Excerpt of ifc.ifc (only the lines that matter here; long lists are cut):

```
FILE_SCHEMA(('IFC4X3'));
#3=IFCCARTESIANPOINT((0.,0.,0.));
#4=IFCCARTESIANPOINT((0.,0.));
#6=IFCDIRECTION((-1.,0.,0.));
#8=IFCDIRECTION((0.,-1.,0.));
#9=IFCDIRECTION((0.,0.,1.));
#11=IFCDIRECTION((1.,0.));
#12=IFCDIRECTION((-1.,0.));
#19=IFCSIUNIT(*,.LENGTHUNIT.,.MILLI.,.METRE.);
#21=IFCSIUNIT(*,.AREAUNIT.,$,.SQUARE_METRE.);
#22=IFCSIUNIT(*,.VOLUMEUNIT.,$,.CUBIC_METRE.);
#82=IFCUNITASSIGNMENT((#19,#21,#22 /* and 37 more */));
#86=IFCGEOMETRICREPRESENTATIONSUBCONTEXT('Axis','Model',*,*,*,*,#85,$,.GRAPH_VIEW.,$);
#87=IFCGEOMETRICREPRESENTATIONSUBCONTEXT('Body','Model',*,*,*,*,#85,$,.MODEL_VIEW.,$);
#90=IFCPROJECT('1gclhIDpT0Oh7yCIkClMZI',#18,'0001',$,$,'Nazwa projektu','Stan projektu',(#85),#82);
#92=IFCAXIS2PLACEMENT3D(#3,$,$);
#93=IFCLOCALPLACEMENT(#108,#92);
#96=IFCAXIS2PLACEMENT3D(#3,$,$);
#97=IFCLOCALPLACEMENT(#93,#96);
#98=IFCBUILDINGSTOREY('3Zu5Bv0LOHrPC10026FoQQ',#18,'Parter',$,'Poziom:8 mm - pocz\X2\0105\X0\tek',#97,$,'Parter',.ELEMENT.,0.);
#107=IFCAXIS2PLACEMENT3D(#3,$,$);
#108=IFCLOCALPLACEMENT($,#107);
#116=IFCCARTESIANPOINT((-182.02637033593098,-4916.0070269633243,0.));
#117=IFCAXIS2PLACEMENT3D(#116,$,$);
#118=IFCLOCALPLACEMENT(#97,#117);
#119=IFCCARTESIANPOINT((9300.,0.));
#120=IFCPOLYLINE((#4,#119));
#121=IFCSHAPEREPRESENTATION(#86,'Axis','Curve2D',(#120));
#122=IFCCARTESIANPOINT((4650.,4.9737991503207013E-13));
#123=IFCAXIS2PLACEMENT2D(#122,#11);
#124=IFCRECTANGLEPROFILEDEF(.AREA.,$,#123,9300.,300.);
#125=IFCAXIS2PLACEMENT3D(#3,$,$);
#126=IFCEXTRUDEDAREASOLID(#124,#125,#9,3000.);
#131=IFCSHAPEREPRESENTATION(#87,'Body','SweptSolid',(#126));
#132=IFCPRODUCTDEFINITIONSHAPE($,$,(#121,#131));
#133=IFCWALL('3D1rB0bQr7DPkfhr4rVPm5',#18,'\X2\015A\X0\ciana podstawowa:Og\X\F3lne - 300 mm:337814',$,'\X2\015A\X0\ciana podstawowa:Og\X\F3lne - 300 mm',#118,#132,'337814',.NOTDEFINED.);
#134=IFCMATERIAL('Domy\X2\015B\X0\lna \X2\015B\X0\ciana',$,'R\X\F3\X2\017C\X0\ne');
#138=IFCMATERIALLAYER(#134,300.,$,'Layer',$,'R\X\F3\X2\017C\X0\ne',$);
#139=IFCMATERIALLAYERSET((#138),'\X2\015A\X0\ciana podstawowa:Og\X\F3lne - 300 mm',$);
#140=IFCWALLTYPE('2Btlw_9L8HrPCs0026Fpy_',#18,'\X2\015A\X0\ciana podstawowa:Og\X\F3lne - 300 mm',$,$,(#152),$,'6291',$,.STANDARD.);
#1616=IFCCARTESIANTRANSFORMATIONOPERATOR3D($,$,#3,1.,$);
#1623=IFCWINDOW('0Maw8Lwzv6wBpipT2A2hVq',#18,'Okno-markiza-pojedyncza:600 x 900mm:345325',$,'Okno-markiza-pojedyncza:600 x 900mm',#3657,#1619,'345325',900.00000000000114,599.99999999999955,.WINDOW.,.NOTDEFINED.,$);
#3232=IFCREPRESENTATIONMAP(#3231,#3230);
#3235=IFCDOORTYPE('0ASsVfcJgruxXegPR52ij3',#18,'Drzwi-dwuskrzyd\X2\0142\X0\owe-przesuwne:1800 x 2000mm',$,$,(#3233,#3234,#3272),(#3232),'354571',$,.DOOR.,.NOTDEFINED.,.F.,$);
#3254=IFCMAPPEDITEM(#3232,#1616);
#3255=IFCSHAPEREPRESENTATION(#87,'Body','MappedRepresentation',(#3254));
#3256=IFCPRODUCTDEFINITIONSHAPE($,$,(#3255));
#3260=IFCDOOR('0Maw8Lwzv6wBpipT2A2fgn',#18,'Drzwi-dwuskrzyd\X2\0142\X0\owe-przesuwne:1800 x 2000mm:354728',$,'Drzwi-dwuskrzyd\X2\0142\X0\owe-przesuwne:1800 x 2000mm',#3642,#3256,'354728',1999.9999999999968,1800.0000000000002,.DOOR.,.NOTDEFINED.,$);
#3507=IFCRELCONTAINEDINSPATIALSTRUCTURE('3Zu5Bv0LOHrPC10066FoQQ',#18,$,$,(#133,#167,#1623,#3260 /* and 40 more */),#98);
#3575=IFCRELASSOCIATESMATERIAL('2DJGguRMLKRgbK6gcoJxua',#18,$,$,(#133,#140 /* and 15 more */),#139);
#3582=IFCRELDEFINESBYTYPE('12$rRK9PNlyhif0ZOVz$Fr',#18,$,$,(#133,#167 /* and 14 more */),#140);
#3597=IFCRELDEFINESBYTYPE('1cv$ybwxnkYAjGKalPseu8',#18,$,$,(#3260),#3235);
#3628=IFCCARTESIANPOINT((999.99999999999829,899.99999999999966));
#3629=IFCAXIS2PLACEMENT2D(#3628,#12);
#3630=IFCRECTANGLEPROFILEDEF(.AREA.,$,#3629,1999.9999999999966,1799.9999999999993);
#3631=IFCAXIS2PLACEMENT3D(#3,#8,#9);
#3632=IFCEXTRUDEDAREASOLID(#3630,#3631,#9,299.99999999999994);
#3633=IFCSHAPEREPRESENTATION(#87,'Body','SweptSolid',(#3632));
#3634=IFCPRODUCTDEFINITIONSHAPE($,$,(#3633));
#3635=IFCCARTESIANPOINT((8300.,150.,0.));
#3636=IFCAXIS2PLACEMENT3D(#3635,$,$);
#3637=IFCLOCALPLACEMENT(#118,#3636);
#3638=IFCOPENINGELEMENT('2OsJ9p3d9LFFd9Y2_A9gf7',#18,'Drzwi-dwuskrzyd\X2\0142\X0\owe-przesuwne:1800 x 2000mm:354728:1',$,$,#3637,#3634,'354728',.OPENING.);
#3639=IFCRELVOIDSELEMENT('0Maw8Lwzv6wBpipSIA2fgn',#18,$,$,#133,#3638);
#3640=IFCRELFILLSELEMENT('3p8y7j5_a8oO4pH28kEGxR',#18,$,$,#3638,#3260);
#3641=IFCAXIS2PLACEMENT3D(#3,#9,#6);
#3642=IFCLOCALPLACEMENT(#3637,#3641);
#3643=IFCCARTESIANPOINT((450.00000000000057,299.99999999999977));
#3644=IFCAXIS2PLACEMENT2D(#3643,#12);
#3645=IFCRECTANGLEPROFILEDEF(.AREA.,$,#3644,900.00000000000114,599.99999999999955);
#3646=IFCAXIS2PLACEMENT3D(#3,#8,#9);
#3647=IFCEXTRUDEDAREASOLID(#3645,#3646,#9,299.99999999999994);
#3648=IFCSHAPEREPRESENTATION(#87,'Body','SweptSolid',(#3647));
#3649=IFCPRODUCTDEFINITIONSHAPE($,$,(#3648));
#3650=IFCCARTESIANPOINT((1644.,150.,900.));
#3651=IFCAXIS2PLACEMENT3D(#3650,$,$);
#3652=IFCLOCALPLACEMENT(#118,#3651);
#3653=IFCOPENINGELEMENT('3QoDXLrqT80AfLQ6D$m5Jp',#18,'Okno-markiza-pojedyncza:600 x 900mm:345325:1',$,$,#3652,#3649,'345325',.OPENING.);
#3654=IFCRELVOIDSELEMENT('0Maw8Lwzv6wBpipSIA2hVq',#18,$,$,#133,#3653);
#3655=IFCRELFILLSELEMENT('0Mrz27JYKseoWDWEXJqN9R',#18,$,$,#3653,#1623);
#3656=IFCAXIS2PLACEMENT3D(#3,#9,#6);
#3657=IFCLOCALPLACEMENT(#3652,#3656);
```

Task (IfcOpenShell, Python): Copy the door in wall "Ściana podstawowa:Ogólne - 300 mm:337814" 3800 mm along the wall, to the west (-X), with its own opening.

```python
import ifcopenshell
import ifcopenshell.api.feature
import ifcopenshell.api.geometry
import ifcopenshell.api.root
import ifcopenshell.geom
import ifcopenshell.util.element
import ifcopenshell.util.placement
import ifcopenshell.util.shape

model = ifcopenshell.open("ifc.ifc")
settings = ifcopenshell.geom.settings()


def volume(element):
    """Net volume in cubic metres, openings subtracted."""
    shape = ifcopenshell.geom.create_shape(settings, element)
    return ifcopenshell.util.shape.get_volume(shape.geometry)


def reuse_history(source, copy):
    """copy_class also copies each property set's owner history, people and application; keep the originals."""
    for rel in copy.IsDefinedBy:
        if rel.is_a("IfcRelDefinesByProperties") and (history := rel.RelatingPropertyDefinition.OwnerHistory):
            rel.RelatingPropertyDefinition.OwnerHistory = source.OwnerHistory
            ifcopenshell.util.element.remove_deep2(model, history)


door = model.by_id(3260)
opening = door.FillsVoids[0].RelatingOpeningElement
wall = opening.VoidsElements[0].RelatingBuildingElement
before = volume(wall)
shift = ifcopenshell.util.placement.get_local_placement(wall.ObjectPlacement)[:3, 0] * -3800.0

# copy_class copies the void relationship, type, container and properties, but no geometry.
new_opening = ifcopenshell.api.root.copy_class(model, product=opening)
new_opening.Representation = ifcopenshell.util.element.copy_deep(
    model, opening.Representation, exclude=["IfcGeometricRepresentationContext", "IfcRepresentationMap"]
)
new_opening.Name = "Drzwi-dwuskrzydłowe-przesuwne:1800 x 2000mm"
new_opening.Tag = None
new_door = ifcopenshell.api.root.copy_class(model, product=door)
new_door.Representation = ifcopenshell.util.element.copy_deep(
    model, door.Representation, exclude=["IfcGeometricRepresentationContext", "IfcRepresentationMap"]
)
new_door.Name = "Drzwi-dwuskrzydłowe-przesuwne:1800 x 2000mm"
new_door.Tag = None
reuse_history(door, new_door)
ifcopenshell.api.feature.add_filling(model, opening=new_opening, element=new_door)

for old, new in ((opening, new_opening), (door, new_door)):
    matrix = ifcopenshell.util.placement.get_local_placement(old.ObjectPlacement)
    matrix[:3, 3] += shift
    ifcopenshell.api.geometry.edit_object_placement(model, product=new, matrix=matrix, is_si=False)

after = volume(wall)

print(f"wall volume {before:.3f} -> {after:.3f} m3")

model.write("ifc-out.ifc")
```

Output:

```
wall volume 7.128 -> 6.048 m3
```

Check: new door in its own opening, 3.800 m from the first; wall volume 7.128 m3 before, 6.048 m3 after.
